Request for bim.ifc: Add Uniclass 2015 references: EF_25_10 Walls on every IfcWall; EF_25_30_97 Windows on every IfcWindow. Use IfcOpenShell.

First a look at what the model holds.

```python
import ifcopenshell

model = ifcopenshell.open("bim.ifc")
print(model.schema)
print("classifications:", [c.Name for c in model.by_type("IfcClassification")])
for ifc_class in ("IfcDoor", "IfcRoof", "IfcStair", "IfcWall", "IfcWindow"):
    print(ifc_class, len(model.by_type(ifc_class)))
```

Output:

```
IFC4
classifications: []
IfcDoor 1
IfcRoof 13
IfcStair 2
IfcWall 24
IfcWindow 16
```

```python
import ifcopenshell
import ifcopenshell.api.classification

model = ifcopenshell.open("bim.ifc")

system = ifcopenshell.api.classification.add_classification(model, classification="Uniclass 2015")

codes = {
    "IfcWall": ("EF_25_10", "Walls"),
    "IfcWindow": ("EF_25_30_97", "Windows"),
}
for ifc_class, (code, name) in codes.items():
    products = model.by_type(ifc_class)
    ifcopenshell.api.classification.add_reference(
        model, products=products, classification=system, identification=code, name=name
    )
    print(code, len(products))

model.write("bim_updated.ifc")
```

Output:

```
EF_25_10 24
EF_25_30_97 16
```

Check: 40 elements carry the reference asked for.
